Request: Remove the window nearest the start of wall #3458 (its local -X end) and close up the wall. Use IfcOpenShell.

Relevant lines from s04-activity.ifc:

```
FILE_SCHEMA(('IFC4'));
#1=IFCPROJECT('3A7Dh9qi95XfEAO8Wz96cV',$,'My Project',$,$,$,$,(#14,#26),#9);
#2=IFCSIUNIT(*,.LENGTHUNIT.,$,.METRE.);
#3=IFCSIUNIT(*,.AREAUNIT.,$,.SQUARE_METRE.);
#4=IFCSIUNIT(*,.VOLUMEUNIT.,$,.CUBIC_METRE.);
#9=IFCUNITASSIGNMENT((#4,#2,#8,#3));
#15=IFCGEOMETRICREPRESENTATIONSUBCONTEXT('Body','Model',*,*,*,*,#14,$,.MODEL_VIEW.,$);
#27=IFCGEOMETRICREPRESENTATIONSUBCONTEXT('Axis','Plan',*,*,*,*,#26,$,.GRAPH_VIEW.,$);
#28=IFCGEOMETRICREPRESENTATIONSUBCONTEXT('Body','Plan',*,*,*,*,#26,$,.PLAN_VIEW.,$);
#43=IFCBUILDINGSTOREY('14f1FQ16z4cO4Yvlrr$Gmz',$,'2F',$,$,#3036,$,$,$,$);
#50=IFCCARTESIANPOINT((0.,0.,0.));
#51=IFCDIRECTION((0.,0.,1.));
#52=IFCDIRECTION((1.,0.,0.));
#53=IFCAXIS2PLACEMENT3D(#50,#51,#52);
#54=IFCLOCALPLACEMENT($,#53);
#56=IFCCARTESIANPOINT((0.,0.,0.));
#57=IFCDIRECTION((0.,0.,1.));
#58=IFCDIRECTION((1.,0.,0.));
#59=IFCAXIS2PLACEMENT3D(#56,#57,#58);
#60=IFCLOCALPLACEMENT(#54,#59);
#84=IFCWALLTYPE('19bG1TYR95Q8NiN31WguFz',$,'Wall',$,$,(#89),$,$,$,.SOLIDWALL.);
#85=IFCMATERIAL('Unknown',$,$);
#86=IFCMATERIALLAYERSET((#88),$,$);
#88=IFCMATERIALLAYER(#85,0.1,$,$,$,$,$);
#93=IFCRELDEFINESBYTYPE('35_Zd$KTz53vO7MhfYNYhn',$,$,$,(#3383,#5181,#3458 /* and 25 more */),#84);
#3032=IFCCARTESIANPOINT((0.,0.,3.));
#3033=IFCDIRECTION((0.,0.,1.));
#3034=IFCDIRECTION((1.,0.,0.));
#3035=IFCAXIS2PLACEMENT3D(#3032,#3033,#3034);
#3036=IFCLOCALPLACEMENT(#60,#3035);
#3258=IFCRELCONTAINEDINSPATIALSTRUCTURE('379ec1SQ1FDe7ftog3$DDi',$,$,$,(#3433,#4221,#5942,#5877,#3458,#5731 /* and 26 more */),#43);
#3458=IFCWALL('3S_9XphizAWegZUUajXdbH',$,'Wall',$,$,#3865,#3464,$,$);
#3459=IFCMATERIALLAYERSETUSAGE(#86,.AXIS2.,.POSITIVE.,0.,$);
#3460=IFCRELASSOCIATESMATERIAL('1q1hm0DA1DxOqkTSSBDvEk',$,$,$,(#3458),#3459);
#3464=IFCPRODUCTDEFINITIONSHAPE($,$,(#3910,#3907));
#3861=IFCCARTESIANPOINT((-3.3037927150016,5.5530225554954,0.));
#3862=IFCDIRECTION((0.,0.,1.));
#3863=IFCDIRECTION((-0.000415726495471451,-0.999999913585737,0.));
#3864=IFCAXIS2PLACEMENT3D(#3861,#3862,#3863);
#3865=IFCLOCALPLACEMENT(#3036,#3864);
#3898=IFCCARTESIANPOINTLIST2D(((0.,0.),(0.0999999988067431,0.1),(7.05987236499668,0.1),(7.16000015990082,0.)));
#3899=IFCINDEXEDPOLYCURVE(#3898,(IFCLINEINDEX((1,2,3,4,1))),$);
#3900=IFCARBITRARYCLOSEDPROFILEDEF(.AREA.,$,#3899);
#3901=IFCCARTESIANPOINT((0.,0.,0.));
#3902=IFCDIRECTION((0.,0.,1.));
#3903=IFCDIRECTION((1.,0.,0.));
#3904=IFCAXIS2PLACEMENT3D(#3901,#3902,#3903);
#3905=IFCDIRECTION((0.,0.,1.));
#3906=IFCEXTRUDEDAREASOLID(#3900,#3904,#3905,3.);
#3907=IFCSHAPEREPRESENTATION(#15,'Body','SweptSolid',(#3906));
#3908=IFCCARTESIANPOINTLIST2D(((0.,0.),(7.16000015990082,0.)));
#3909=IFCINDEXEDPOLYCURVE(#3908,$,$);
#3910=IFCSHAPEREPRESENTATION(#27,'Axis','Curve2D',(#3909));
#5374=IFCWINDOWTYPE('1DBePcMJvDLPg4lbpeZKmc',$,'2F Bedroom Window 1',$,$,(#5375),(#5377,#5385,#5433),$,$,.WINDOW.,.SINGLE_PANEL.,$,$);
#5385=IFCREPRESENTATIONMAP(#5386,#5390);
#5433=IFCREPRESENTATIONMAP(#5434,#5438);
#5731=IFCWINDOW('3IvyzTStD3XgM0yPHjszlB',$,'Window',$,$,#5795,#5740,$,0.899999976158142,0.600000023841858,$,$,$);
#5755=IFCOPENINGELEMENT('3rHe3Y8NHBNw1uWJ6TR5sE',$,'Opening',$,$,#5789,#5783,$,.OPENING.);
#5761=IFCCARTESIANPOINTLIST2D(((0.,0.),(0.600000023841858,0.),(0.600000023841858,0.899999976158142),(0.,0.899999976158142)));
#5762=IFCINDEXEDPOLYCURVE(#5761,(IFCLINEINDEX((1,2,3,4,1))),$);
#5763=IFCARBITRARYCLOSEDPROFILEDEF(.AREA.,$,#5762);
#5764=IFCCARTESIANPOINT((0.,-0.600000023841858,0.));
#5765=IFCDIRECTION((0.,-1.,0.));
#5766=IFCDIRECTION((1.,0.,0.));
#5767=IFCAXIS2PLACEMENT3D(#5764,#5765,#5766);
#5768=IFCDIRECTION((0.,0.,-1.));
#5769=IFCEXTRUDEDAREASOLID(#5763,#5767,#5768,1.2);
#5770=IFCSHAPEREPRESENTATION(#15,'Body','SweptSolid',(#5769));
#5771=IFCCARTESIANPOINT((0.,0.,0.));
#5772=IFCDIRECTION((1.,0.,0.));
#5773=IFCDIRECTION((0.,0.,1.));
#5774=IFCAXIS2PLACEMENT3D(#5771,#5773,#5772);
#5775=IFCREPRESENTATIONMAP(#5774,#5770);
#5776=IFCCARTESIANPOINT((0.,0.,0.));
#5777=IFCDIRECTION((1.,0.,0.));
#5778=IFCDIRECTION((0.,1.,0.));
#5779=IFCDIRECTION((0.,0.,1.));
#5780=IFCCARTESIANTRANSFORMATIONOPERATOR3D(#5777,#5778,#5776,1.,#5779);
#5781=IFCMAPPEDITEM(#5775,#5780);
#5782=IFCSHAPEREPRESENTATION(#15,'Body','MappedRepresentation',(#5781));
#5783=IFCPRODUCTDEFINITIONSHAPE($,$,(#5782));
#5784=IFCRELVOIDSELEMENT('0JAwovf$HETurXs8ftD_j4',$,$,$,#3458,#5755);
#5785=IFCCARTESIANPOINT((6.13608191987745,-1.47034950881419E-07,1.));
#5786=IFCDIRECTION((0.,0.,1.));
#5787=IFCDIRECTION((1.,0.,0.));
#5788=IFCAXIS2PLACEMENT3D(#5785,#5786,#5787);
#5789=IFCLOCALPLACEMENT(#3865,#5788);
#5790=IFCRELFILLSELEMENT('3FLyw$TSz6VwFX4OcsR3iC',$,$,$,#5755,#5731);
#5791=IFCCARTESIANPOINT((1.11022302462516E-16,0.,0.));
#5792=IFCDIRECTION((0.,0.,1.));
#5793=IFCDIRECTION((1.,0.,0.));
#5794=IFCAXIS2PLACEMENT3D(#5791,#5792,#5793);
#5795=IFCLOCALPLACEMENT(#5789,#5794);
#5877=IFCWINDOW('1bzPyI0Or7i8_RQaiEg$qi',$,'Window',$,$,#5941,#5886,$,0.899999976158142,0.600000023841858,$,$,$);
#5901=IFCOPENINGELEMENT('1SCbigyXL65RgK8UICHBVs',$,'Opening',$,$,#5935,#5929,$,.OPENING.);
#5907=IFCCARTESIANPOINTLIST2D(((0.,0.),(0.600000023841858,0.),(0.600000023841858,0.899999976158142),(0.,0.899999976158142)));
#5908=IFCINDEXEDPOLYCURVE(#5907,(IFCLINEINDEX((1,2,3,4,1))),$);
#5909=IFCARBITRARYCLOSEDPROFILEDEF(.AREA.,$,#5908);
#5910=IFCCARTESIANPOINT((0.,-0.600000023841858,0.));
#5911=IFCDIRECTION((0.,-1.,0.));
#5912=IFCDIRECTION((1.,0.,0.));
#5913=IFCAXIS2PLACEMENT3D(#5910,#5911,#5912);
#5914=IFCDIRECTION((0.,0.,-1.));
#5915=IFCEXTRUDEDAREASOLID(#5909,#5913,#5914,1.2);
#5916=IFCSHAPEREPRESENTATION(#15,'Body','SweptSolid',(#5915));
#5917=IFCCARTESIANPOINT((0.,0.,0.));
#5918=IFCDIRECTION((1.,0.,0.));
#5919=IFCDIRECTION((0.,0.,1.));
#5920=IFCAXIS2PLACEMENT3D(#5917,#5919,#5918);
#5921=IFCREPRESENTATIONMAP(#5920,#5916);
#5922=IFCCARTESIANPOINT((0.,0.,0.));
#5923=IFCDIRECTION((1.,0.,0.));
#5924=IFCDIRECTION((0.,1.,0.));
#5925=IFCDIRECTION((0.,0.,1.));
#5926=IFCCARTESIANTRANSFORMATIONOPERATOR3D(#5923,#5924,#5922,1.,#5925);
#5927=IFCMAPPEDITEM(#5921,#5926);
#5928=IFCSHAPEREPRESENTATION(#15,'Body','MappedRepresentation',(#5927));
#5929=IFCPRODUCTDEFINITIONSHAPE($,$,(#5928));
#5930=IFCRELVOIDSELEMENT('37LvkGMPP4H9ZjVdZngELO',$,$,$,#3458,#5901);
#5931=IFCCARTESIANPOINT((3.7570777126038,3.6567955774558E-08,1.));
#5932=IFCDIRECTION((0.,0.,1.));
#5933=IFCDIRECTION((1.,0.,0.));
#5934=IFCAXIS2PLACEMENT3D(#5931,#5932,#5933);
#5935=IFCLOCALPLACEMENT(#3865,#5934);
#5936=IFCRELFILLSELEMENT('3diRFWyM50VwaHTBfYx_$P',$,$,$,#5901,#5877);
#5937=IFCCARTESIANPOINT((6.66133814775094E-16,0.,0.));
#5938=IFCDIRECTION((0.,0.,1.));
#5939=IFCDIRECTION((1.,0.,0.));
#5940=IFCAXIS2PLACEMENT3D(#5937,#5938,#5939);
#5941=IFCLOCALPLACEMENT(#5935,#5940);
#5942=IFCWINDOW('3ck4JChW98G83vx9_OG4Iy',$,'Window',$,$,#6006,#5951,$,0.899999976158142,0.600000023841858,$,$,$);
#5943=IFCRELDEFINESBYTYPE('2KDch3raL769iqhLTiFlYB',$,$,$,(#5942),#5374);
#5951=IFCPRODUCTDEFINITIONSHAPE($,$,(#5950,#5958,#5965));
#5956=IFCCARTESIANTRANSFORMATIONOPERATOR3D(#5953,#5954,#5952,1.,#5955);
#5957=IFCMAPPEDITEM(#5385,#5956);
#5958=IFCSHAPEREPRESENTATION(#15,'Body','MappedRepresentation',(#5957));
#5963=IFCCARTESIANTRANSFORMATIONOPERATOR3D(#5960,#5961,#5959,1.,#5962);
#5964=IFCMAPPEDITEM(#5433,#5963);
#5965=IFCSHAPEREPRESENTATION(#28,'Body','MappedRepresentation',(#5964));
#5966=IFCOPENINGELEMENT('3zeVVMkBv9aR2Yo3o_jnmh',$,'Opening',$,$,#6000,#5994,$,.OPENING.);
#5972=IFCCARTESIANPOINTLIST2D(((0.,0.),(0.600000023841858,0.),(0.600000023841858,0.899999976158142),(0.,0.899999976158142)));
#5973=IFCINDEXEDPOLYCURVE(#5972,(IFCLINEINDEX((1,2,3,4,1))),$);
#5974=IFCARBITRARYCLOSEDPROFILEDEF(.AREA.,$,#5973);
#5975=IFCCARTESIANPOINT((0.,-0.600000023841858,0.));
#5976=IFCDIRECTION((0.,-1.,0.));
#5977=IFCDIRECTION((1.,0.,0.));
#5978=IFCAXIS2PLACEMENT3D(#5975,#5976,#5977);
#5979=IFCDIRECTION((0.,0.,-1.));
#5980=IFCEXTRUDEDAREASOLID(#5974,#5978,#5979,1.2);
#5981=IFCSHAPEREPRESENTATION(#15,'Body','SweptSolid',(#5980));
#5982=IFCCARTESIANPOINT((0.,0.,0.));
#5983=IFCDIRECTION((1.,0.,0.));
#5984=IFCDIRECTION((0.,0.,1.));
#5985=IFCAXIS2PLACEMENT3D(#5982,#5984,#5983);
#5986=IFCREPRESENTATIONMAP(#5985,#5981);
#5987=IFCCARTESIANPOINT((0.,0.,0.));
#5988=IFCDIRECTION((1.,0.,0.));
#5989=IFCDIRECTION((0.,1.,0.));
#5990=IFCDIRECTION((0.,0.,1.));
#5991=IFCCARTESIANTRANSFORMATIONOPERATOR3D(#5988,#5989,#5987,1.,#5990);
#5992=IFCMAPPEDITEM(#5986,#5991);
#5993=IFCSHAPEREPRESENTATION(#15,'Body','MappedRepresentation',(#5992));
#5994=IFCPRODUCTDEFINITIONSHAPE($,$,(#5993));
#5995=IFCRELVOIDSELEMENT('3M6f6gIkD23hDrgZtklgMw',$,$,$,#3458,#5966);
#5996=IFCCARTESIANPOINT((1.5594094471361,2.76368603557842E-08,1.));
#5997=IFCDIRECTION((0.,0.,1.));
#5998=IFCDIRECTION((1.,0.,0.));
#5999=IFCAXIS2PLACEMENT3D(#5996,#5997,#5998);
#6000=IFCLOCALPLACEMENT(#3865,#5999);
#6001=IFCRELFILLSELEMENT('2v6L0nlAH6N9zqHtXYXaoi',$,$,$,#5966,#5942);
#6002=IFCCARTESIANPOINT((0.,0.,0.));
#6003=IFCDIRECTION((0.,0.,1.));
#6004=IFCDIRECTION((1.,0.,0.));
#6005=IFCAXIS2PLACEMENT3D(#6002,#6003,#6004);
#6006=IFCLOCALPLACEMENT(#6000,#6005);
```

```python
import ifcopenshell
import ifcopenshell.api.feature
import ifcopenshell.api.root
import ifcopenshell.geom
import ifcopenshell.util.shape

model = ifcopenshell.open("s04-activity.ifc")
settings = ifcopenshell.geom.settings()


def volume(element):
    """Net volume in cubic metres, openings subtracted."""
    shape = ifcopenshell.geom.create_shape(settings, element)
    return ifcopenshell.util.shape.get_volume(shape.geometry)


window = model.by_guid("3ck4JChW98G83vx9_OG4Iy")
opening = window.FillsVoids[0].RelatingOpeningElement
wall = opening.VoidsElements[0].RelatingBuildingElement
before = volume(wall)

ifcopenshell.api.root.remove_product(model, product=window)
ifcopenshell.api.feature.remove_feature(model, feature=opening)

after = volume(wall)

print(f"wall volume {before:.3f} -> {after:.3f} m3")

model.write("s04-activity_updated.ifc")
```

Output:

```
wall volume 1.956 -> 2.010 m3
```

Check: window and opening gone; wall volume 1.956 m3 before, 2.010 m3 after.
